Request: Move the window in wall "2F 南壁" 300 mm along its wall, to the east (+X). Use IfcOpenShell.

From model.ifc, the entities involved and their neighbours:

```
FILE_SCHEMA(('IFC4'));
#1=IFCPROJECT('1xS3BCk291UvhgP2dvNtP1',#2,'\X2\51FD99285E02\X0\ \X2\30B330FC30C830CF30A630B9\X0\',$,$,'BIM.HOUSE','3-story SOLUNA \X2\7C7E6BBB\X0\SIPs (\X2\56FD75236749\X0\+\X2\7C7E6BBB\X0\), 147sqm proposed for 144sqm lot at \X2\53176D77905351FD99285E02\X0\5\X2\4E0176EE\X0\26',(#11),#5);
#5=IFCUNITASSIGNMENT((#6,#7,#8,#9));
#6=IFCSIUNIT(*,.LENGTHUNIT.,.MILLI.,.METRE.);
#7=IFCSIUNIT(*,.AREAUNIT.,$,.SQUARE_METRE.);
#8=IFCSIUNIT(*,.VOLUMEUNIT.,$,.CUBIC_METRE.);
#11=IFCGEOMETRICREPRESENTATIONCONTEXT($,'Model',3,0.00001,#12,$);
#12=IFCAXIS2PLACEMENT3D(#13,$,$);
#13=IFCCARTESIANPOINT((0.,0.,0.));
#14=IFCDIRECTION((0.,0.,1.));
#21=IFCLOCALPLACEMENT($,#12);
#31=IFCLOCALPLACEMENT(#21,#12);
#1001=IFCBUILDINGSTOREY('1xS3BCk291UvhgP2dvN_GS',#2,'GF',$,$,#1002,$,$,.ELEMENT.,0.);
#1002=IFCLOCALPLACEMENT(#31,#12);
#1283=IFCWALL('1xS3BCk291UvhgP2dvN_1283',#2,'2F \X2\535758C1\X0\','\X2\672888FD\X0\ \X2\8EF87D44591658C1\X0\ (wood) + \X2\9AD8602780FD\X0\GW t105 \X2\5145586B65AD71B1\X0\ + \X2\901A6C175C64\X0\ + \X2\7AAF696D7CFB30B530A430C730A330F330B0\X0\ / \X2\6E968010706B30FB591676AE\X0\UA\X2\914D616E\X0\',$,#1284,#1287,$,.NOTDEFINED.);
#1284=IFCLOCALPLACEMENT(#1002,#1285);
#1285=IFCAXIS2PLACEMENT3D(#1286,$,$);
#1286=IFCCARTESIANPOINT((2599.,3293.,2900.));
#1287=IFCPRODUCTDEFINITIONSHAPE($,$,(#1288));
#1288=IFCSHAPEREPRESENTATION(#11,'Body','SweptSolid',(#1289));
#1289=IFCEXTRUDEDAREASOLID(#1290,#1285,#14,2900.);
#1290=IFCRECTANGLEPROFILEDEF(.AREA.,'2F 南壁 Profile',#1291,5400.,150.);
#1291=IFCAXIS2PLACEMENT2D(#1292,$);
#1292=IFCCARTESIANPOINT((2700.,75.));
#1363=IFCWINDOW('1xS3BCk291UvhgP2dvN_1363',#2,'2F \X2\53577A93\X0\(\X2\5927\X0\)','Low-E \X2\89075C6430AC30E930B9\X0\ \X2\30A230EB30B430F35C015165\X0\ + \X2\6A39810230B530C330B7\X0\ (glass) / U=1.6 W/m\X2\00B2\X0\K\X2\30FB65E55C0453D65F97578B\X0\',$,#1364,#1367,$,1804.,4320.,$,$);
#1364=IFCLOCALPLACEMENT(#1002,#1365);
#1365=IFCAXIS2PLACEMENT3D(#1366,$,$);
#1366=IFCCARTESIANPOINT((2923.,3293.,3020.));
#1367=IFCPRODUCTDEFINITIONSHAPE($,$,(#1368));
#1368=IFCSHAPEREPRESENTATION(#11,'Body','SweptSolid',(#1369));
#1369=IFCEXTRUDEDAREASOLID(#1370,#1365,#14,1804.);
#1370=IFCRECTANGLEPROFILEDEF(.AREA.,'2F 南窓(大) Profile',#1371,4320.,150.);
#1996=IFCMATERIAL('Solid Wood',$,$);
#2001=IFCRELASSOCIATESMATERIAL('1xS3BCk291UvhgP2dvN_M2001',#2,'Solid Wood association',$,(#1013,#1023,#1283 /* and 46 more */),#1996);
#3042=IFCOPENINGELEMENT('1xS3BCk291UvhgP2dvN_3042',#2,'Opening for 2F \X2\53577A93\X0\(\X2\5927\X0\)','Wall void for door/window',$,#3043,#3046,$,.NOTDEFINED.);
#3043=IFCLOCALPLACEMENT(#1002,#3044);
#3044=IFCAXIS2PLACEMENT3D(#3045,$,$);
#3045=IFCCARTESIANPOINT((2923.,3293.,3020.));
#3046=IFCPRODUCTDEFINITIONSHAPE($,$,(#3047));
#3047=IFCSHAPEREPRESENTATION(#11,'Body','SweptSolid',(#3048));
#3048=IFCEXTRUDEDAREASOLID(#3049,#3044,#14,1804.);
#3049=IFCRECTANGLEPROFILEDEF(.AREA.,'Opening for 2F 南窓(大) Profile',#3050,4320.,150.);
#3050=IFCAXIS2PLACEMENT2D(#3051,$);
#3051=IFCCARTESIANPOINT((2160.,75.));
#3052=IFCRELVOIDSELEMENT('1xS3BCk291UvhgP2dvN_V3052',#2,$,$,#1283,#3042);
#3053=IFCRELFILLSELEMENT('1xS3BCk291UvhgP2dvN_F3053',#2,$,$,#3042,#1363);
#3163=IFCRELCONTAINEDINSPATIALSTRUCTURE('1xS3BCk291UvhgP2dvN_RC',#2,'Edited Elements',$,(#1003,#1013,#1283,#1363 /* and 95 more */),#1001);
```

```python
import ifcopenshell
import ifcopenshell.api.geometry
import ifcopenshell.util.placement
import ifcopenshell.util.unit

model = ifcopenshell.open("model.ifc")
unit_scale = ifcopenshell.util.unit.calculate_unit_scale(model)

window = model.by_guid("1xS3BCk291UvhgP2dvN_1363")
opening = window.FillsVoids[0].RelatingOpeningElement
wall = opening.VoidsElements[0].RelatingBuildingElement

wall_matrix = ifcopenshell.util.placement.get_local_placement(wall.ObjectPlacement)
shift = wall_matrix[:3, 0] * 0.3 / unit_scale
before = ifcopenshell.util.placement.get_local_placement(window.ObjectPlacement)[:3, 3].copy()

# The window is not placed relative to its opening, so move both.
for product in (opening, window):
    matrix = ifcopenshell.util.placement.get_local_placement(product.ObjectPlacement)
    matrix[:3, 3] += shift
    ifcopenshell.api.geometry.edit_object_placement(model, product=product, matrix=matrix, is_si=False)

after = ifcopenshell.util.placement.get_local_placement(window.ObjectPlacement)[:3, 3]
print("window moved by", (after - before).round(3) + 0.0)

model.write("model_edited.ifc")
```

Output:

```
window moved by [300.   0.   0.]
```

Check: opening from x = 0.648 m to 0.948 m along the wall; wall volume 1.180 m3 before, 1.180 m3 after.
